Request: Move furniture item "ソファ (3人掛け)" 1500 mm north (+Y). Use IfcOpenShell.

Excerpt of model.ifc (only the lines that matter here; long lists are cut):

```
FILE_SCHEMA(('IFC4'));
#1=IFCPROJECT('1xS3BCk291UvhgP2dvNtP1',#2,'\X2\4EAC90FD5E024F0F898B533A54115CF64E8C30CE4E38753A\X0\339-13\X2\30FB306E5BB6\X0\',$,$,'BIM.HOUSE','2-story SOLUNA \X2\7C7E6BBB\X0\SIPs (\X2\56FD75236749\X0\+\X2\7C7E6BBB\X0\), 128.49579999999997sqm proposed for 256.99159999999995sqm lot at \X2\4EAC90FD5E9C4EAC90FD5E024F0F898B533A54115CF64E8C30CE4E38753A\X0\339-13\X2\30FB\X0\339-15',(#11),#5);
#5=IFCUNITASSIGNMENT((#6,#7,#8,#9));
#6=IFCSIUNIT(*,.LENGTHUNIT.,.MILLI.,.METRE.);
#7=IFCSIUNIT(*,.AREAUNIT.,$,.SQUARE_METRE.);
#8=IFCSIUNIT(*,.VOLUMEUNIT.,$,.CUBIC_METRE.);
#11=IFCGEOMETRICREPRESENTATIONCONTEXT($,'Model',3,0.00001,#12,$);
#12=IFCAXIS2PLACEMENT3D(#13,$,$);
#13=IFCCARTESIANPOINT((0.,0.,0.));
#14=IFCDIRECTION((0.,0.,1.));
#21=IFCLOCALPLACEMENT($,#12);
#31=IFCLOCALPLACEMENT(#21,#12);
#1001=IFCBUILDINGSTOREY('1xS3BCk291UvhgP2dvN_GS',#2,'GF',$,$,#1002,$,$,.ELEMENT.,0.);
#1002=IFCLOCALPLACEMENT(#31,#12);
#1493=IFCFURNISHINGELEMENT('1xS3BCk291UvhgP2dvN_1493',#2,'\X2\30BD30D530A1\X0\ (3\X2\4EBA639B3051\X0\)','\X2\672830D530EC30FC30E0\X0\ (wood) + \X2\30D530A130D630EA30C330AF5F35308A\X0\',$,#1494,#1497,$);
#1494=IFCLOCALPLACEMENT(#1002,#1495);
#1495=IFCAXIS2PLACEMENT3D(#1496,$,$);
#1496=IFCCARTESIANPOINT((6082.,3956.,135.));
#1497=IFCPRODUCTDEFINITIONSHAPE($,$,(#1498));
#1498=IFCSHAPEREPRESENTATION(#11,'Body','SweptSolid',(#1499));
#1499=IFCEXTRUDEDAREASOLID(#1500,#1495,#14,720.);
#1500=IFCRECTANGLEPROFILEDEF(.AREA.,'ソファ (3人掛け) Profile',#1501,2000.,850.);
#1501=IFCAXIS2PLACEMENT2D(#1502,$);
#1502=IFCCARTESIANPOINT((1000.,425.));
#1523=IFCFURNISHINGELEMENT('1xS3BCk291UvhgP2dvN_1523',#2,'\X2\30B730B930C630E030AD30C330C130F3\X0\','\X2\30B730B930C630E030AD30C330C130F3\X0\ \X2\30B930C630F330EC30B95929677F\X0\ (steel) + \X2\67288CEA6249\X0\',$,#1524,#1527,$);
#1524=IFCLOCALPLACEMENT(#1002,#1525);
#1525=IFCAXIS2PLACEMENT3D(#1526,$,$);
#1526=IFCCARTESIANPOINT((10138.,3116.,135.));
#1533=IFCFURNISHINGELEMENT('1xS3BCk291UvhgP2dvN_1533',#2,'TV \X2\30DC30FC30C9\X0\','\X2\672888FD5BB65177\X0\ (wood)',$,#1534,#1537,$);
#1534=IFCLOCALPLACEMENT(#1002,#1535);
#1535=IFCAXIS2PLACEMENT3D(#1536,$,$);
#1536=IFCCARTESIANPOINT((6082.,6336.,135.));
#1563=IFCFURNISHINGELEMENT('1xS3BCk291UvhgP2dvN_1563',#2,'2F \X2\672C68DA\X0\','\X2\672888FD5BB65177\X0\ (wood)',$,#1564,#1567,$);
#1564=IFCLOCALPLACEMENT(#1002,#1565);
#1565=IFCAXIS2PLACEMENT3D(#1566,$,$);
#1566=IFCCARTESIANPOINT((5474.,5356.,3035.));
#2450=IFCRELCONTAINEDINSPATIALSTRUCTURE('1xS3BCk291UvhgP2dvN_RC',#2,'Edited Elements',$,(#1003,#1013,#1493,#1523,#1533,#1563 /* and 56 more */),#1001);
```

```python
import ifcopenshell
import ifcopenshell.api.geometry
import ifcopenshell.util.placement
import ifcopenshell.util.unit

model = ifcopenshell.open("model.ifc")
unit_scale = ifcopenshell.util.unit.calculate_unit_scale(model)

item = model.by_guid("1xS3BCk291UvhgP2dvN_1493")
matrix = ifcopenshell.util.placement.get_local_placement(item.ObjectPlacement)
matrix[1, 3] += 1.5 / unit_scale
ifcopenshell.api.geometry.edit_object_placement(model, product=item, matrix=matrix, is_si=False)

print(ifcopenshell.util.placement.get_local_placement(item.ObjectPlacement).round(3) + 0.0)

model.write("model-out.ifc")
```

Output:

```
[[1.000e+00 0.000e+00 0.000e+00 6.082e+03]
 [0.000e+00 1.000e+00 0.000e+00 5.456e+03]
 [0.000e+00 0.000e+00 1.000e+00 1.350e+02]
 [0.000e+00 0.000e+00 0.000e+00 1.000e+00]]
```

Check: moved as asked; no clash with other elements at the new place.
